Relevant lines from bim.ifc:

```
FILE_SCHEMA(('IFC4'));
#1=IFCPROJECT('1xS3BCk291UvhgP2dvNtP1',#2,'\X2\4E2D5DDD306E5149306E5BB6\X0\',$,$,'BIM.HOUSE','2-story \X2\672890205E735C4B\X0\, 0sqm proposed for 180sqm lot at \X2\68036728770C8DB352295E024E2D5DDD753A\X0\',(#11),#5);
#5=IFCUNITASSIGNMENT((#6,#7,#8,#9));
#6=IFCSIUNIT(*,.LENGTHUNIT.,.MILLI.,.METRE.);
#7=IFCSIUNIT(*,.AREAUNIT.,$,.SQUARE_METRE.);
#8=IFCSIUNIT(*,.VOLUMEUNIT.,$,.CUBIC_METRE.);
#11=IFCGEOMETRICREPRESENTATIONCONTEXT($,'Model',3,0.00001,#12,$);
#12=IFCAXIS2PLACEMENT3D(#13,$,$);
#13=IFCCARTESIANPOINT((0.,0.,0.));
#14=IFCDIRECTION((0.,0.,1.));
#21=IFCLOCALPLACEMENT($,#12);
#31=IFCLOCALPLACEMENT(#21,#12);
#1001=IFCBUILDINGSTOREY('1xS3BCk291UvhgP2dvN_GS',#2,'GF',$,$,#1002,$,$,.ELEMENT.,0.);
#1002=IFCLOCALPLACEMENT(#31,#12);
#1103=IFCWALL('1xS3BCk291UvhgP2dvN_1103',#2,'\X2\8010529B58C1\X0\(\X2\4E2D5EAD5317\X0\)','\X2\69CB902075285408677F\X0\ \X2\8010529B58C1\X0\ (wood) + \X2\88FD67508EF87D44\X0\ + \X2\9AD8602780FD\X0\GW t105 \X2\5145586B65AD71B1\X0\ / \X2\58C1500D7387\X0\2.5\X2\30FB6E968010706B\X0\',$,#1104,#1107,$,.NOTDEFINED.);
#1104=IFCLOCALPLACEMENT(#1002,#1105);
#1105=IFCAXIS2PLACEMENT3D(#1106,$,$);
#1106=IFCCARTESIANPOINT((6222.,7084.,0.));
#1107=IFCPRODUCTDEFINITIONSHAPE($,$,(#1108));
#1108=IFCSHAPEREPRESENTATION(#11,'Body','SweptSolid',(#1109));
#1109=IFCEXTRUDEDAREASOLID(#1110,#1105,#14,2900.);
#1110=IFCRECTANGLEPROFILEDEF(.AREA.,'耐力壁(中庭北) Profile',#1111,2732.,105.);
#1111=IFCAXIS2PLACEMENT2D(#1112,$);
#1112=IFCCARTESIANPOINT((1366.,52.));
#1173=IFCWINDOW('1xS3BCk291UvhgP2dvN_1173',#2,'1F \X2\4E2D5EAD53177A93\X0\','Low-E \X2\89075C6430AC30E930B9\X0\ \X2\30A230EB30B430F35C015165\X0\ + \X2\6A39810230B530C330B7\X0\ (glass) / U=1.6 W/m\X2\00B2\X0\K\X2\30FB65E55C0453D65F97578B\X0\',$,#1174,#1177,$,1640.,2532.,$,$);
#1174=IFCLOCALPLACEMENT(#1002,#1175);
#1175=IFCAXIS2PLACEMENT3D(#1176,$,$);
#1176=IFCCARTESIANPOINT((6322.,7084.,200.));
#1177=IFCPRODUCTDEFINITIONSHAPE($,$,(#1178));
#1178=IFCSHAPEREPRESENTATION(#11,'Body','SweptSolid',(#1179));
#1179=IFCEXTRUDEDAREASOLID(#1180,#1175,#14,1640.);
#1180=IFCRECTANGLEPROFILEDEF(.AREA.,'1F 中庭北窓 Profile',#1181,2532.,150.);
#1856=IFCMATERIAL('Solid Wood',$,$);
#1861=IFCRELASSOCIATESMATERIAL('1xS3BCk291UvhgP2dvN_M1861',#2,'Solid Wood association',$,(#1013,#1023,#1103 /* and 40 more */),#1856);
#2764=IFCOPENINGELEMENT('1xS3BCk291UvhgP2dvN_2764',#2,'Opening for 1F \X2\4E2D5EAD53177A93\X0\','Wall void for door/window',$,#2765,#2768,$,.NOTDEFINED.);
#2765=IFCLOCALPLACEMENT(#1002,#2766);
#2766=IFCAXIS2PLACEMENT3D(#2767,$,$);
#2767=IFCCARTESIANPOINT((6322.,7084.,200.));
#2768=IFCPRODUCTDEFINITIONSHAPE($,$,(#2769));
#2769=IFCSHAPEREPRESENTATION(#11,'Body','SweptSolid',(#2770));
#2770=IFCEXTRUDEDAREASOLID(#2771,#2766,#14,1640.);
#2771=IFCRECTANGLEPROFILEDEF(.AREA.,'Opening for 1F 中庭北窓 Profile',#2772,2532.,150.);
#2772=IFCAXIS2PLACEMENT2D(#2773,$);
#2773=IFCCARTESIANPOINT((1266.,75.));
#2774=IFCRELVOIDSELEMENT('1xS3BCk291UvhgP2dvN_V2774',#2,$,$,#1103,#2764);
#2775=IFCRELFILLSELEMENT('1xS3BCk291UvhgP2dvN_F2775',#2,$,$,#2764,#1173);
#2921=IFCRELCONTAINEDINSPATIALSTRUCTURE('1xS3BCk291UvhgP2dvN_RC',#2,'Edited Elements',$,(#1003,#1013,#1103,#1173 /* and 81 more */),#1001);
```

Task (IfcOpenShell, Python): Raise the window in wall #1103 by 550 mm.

```python
import numpy as np
import ifcopenshell
import ifcopenshell.api.geometry
import ifcopenshell.util.placement
import ifcopenshell.util.unit

model = ifcopenshell.open("bim.ifc")
unit_scale = ifcopenshell.util.unit.calculate_unit_scale(model)

window = model.by_guid("1xS3BCk291UvhgP2dvN_1173")
opening = window.FillsVoids[0].RelatingOpeningElement
dz = 0.55 / unit_scale

shift = np.array([0.0, 0.0, dz])
# The window is not placed relative to its opening, so move both.
for product in (opening, window):
    matrix = ifcopenshell.util.placement.get_local_placement(product.ObjectPlacement)
    matrix[:3, 3] += shift
    ifcopenshell.api.geometry.edit_object_placement(model, product=product, matrix=matrix, is_si=False)

print(f"moved by {dz * unit_scale:+.3f} m")

model.write("bim_rev.ifc")
```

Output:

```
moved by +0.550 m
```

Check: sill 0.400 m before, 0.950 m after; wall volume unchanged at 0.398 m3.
